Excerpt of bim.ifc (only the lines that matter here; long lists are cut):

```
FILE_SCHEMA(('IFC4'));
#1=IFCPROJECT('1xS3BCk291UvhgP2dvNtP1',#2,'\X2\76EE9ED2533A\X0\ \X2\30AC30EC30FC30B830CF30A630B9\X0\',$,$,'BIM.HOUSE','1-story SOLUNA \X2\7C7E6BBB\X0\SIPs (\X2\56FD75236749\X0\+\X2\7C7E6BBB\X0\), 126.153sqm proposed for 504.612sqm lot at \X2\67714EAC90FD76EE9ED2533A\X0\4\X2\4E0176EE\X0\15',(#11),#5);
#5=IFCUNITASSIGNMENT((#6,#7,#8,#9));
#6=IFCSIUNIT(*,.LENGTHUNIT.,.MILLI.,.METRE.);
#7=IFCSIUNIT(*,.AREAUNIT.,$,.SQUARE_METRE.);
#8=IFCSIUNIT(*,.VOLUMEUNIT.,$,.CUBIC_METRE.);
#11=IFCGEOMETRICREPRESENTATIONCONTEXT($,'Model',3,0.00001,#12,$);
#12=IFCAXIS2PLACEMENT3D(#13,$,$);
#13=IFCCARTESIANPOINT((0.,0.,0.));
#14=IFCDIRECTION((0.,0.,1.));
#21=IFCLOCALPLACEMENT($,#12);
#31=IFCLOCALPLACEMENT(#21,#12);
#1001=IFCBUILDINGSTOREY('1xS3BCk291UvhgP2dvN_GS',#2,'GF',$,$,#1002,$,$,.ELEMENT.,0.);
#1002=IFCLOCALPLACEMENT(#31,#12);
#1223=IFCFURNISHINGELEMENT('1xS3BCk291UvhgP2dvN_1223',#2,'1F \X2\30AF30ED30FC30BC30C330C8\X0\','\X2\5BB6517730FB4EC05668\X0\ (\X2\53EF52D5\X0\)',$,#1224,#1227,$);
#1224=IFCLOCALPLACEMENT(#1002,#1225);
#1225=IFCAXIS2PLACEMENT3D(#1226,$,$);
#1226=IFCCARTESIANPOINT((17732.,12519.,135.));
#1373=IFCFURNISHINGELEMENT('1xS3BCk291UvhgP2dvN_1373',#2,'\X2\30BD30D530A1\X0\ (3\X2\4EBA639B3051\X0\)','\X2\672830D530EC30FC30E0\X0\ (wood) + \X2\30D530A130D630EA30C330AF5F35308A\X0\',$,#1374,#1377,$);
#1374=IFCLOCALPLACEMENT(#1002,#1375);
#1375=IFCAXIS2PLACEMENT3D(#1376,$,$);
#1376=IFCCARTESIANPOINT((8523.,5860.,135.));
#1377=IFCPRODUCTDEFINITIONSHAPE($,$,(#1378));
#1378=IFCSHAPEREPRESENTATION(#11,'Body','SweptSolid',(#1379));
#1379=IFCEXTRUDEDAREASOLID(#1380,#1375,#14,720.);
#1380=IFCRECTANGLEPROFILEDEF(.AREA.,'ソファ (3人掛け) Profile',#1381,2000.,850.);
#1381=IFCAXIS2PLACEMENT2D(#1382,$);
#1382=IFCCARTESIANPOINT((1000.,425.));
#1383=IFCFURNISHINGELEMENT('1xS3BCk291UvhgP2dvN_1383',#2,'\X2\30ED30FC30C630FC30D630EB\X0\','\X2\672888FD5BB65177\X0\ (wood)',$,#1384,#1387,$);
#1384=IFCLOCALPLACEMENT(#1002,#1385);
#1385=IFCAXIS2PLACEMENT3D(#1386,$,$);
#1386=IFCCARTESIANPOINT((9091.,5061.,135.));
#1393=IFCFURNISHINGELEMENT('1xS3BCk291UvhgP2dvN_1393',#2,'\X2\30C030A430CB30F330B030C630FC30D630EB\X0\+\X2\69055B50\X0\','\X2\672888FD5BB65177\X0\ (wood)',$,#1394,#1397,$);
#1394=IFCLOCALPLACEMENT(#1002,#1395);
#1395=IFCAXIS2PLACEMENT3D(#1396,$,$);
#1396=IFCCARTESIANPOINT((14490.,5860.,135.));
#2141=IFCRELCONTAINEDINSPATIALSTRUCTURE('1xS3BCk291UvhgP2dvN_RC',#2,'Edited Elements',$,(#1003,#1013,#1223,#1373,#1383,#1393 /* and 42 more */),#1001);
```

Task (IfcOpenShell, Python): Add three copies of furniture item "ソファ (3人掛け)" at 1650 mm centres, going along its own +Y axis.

```python
import ifcopenshell
import ifcopenshell.api.geometry
import ifcopenshell.api.root
import ifcopenshell.util.element
import ifcopenshell.util.placement
import ifcopenshell.util.unit

model = ifcopenshell.open("bim.ifc")
unit_scale = ifcopenshell.util.unit.calculate_unit_scale(model)


def reuse_history(source, copy):
    """copy_class also copies each property set's owner history, people and application; keep the originals."""
    for rel in copy.IsDefinedBy:
        if rel.is_a("IfcRelDefinesByProperties") and (history := rel.RelatingPropertyDefinition.OwnerHistory):
            rel.RelatingPropertyDefinition.OwnerHistory = source.OwnerHistory
            ifcopenshell.util.element.remove_deep2(model, history)


source = model.by_id(1373)
base = ifcopenshell.util.placement.get_local_placement(source.ObjectPlacement)
step = base[:3, 1] * 1.65 / unit_scale

for i in range(1, 4):
    copy = ifcopenshell.api.root.copy_class(model, product=source)
    copy.Representation = ifcopenshell.util.element.copy_deep(
        model, source.Representation, exclude=["IfcGeometricRepresentationContext", "IfcRepresentationMap"]
    )
    reuse_history(source, copy)
    matrix = base.copy()
    matrix[:3, 3] += i * step
    print("added at", matrix[:3, 3].round(3) + 0.0)
    ifcopenshell.api.geometry.edit_object_placement(model, product=copy, matrix=matrix, is_si=False)

model.write("bim_rev.ifc")
```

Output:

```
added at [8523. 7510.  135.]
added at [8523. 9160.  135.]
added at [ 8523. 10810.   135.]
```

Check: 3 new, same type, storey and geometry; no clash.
